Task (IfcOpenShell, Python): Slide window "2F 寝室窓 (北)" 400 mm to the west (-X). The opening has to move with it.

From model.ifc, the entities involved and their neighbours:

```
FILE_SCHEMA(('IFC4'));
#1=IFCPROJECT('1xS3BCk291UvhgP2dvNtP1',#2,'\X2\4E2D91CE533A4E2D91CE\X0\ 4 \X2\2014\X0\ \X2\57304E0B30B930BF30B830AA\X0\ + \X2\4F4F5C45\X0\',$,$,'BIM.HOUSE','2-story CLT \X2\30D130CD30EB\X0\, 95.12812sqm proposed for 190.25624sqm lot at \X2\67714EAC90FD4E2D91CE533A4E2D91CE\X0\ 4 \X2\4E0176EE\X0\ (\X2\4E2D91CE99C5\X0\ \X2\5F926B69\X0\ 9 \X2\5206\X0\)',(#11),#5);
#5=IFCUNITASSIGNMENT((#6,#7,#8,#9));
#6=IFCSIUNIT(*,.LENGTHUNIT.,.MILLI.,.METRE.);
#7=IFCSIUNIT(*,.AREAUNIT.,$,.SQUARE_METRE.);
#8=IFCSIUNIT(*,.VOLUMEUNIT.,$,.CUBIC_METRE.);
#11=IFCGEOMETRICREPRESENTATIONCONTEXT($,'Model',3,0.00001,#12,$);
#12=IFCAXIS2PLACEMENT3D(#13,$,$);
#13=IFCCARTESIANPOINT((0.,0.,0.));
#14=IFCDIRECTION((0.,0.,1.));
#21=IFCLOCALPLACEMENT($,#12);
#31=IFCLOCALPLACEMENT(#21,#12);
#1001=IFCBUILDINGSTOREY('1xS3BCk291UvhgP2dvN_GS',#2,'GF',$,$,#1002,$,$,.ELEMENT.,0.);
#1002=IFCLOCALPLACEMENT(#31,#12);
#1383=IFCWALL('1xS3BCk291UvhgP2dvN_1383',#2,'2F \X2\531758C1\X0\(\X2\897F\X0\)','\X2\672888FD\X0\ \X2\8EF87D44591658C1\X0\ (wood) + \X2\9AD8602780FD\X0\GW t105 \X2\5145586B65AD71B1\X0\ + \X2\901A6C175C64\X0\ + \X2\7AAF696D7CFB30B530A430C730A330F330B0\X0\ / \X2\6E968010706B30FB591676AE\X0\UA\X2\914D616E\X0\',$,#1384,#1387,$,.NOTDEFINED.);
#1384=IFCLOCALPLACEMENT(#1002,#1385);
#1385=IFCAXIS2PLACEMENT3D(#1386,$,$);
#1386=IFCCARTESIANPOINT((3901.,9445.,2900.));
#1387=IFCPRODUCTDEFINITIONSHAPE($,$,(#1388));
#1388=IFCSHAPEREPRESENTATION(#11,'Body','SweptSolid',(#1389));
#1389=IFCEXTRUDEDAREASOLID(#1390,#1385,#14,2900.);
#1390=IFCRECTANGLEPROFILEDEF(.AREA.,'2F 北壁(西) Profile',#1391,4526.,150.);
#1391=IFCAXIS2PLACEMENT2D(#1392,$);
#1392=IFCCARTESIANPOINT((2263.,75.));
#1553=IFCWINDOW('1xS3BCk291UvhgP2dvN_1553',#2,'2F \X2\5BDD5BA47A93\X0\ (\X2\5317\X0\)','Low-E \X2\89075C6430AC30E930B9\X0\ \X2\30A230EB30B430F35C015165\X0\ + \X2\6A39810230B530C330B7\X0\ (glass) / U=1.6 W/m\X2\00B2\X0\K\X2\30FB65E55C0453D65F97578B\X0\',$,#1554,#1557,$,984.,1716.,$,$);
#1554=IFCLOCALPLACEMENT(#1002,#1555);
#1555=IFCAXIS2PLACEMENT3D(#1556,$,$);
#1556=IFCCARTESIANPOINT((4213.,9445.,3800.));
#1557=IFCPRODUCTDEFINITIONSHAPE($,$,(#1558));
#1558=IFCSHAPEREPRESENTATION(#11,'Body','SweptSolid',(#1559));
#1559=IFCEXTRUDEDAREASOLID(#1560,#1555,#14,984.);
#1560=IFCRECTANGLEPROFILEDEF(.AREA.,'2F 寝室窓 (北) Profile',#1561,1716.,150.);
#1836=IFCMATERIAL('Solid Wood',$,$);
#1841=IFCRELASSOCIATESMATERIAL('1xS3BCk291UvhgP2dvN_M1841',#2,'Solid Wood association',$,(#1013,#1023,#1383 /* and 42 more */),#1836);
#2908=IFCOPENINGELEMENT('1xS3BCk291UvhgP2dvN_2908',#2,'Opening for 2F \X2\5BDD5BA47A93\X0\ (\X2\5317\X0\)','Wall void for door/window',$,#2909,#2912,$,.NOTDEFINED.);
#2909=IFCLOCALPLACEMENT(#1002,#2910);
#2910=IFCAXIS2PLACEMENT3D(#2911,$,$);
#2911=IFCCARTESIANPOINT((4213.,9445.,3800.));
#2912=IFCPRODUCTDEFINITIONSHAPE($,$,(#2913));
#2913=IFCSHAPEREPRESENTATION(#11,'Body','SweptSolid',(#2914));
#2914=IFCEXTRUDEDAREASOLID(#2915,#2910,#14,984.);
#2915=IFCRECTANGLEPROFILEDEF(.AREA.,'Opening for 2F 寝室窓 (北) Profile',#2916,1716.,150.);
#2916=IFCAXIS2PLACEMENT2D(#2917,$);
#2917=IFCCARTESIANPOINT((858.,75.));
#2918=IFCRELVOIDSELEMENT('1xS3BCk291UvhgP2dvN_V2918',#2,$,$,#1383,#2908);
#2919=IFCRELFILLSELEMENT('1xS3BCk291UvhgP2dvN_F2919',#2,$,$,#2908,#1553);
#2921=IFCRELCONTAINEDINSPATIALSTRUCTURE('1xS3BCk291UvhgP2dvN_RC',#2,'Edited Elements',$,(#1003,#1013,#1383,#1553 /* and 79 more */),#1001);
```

```python
import ifcopenshell
import ifcopenshell.api.geometry
import ifcopenshell.util.placement

model = ifcopenshell.open("model.ifc")

window = model.by_guid("1xS3BCk291UvhgP2dvN_1553")
opening = window.FillsVoids[0].RelatingOpeningElement
wall = opening.VoidsElements[0].RelatingBuildingElement

wall_matrix = ifcopenshell.util.placement.get_local_placement(wall.ObjectPlacement)
shift = wall_matrix[:3, 0] * -400.0
before = ifcopenshell.util.placement.get_local_placement(window.ObjectPlacement)[:3, 3].copy()

# The window is not placed relative to its opening, so move both.
for product in (opening, window):
    matrix = ifcopenshell.util.placement.get_local_placement(product.ObjectPlacement)
    matrix[:3, 3] += shift
    ifcopenshell.api.geometry.edit_object_placement(model, product=product, matrix=matrix, is_si=False)

after = ifcopenshell.util.placement.get_local_placement(window.ObjectPlacement)[:3, 3]
print("window moved by", (after - before).round(3) + 0.0)

model.write("model_rev.ifc")
```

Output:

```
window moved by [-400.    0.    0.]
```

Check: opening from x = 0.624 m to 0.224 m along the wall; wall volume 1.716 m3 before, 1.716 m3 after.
